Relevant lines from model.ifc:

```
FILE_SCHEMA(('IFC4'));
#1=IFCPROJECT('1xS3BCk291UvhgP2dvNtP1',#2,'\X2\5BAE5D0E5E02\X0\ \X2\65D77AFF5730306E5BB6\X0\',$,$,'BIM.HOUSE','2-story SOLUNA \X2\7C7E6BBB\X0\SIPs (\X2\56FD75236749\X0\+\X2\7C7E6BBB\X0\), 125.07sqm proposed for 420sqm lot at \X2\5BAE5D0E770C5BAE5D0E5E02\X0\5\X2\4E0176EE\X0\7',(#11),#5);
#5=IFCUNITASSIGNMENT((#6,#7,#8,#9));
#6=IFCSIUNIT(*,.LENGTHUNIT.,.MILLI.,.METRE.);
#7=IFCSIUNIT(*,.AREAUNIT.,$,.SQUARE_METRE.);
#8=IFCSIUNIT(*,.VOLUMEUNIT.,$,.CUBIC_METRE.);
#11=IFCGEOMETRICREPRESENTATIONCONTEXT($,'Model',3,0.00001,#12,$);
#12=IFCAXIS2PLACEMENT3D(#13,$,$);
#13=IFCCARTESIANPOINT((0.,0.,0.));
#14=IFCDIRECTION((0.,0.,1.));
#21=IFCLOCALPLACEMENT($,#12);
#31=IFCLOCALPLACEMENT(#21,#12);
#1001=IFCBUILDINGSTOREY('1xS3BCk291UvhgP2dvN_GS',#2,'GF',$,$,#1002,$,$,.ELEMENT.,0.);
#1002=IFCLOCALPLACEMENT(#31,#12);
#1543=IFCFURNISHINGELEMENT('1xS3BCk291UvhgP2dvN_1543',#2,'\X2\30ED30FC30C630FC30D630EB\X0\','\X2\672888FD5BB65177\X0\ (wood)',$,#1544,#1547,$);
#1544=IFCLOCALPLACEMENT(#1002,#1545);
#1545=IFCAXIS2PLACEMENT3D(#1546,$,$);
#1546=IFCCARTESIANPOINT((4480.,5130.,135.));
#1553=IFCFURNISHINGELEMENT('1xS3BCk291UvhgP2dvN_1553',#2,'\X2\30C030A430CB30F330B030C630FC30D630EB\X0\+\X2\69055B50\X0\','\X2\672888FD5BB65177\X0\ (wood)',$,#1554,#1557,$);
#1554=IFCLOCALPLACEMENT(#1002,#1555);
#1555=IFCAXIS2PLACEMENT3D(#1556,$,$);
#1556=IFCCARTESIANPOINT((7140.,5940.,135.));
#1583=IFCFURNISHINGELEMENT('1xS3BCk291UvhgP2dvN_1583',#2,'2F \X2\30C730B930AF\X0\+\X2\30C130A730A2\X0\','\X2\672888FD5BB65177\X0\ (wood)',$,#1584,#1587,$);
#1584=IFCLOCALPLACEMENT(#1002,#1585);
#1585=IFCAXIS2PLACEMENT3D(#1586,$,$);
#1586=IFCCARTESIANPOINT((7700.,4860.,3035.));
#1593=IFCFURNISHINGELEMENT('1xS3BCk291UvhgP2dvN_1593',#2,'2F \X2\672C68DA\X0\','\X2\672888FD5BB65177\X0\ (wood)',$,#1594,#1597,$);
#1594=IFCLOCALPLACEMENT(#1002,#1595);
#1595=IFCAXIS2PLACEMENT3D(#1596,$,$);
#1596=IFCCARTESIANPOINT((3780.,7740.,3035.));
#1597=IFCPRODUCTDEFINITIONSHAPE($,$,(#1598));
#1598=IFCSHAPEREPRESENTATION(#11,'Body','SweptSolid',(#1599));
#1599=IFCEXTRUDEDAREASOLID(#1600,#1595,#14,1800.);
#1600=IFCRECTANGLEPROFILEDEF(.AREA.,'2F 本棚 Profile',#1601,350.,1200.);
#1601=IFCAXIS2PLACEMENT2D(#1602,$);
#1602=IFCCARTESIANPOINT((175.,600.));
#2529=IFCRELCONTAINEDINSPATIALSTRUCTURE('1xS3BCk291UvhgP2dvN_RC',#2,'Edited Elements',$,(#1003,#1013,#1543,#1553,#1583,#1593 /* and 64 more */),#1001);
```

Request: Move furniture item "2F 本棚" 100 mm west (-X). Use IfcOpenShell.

```python
import ifcopenshell
import ifcopenshell.api.geometry
import ifcopenshell.util.placement
import ifcopenshell.util.unit

model = ifcopenshell.open("model.ifc")
unit_scale = ifcopenshell.util.unit.calculate_unit_scale(model)

item = model.by_guid("1xS3BCk291UvhgP2dvN_1593")
matrix = ifcopenshell.util.placement.get_local_placement(item.ObjectPlacement)
matrix[0, 3] -= 0.1 / unit_scale
ifcopenshell.api.geometry.edit_object_placement(model, product=item, matrix=matrix, is_si=False)

print(ifcopenshell.util.placement.get_local_placement(item.ObjectPlacement).round(3) + 0.0)

model.write("model_edited.ifc")
```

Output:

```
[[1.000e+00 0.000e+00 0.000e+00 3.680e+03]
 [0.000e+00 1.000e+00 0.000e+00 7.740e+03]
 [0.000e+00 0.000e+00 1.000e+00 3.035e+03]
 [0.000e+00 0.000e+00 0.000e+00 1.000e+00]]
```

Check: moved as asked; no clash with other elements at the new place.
